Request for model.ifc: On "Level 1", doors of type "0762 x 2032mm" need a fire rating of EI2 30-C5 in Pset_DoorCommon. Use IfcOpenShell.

First a look at what the model holds.

```python
import ifcopenshell
import ifcopenshell.util.element

model = ifcopenshell.open("model.ifc")
print(model.schema)
storey = next(s for s in model.by_type("IfcBuildingStorey") if s.Name == "Level 1")
doors = [e for e in ifcopenshell.util.element.get_decomposition(storey) if e.is_a("IfcDoor")]
seen = {}
for e in doors:
    element_type = ifcopenshell.util.element.get_type(e)
    key = (element_type.Name if element_type != e and element_type else None, ifcopenshell.util.element.get_pset(e, "Pset_DoorCommon", "FireRating"))
    seen[key] = seen.get(key, 0) + 1
for (name, value), count in sorted(seen.items(), key=str):
    print(count, "x", name, "|", value)
```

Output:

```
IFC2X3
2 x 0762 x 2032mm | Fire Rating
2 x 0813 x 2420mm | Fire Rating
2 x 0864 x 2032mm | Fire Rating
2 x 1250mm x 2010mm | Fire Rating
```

```python
import ifcopenshell
import ifcopenshell.api.pset
import ifcopenshell.util.element

model = ifcopenshell.open("model.ifc")

storey = next(s for s in model.by_type("IfcBuildingStorey") if s.Name == "Level 1")
doors = [e for e in ifcopenshell.util.element.get_decomposition(storey) if e.is_a("IfcDoor")]

count = 0
for e in doors:
    element_type = ifcopenshell.util.element.get_type(e)
    if element_type in (None, e) or element_type.Name != "0762 x 2032mm":
        continue
    # add_pset returns the element's existing set when there is one.
    pset = ifcopenshell.api.pset.add_pset(model, product=e, name="Pset_DoorCommon")
    ifcopenshell.api.pset.edit_pset(model, pset=pset, properties={"FireRating": "EI2 30-C5"})
    count += 1

print(count, "doors updated")

model.write("model_v2.ifc")
```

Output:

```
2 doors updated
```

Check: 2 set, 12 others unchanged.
